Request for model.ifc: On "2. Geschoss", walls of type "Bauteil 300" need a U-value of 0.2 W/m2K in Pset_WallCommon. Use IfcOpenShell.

First a look at what the model holds.

```python
import ifcopenshell
import ifcopenshell.util.element

model = ifcopenshell.open("model.ifc")
print(model.schema)
storey = next(s for s in model.by_type("IfcBuildingStorey") if s.Name == "2. Geschoss")
walls = [e for e in ifcopenshell.util.element.get_decomposition(storey) if e.is_a("IfcWall")]
seen = {}
for e in walls:
    element_type = ifcopenshell.util.element.get_type(e)
    key = (element_type.Name if element_type != e and element_type else None, ifcopenshell.util.element.get_pset(e, "Pset_WallCommon", "ThermalTransmittance"))
    seen[key] = seen.get(key, 0) + 1
for (name, value), count in sorted(seen.items(), key=str):
    print(count, "x", name, "|", value)
```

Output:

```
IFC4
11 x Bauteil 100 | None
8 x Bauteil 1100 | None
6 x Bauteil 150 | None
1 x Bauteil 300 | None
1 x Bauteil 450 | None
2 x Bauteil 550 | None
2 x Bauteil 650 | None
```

```python
import ifcopenshell
import ifcopenshell.api.pset
import ifcopenshell.util.element

model = ifcopenshell.open("model.ifc")

storey = next(s for s in model.by_type("IfcBuildingStorey") if s.Name == "2. Geschoss")
walls = [e for e in ifcopenshell.util.element.get_decomposition(storey) if e.is_a("IfcWall")]

count = 0
for e in walls:
    element_type = ifcopenshell.util.element.get_type(e)
    if element_type in (None, e) or element_type.Name != "Bauteil 300":
        continue
    # add_pset returns the element's existing set when there is one.
    pset = ifcopenshell.api.pset.add_pset(model, product=e, name="Pset_WallCommon")
    ifcopenshell.api.pset.edit_pset(model, pset=pset, properties={"ThermalTransmittance": 0.2})
    count += 1

print(count, "walls updated")

model.write("model_rev.ifc")
```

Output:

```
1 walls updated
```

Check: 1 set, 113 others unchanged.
